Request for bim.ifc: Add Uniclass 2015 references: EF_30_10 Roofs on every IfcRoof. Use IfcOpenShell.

First a look at what the model holds.

```python
import ifcopenshell

model = ifcopenshell.open("bim.ifc")
print(model.schema)
print("classifications:", [c.Name for c in model.by_type("IfcClassification")])
for ifc_class in ("IfcDoor", "IfcRoof", "IfcStair", "IfcWall", "IfcWindow"):
    print(ifc_class, len(model.by_type(ifc_class)))
```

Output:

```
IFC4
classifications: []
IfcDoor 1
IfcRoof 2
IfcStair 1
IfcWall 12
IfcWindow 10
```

```python
import ifcopenshell
import ifcopenshell.api.classification

model = ifcopenshell.open("bim.ifc")

system = ifcopenshell.api.classification.add_classification(model, classification="Uniclass 2015")

codes = {
    "IfcRoof": ("EF_30_10", "Roofs"),
}
for ifc_class, (code, name) in codes.items():
    products = model.by_type(ifc_class)
    ifcopenshell.api.classification.add_reference(
        model, products=products, classification=system, identification=code, name=name
    )
    print(code, len(products))

model.write("bim_v2.ifc")
```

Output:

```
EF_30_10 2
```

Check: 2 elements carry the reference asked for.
